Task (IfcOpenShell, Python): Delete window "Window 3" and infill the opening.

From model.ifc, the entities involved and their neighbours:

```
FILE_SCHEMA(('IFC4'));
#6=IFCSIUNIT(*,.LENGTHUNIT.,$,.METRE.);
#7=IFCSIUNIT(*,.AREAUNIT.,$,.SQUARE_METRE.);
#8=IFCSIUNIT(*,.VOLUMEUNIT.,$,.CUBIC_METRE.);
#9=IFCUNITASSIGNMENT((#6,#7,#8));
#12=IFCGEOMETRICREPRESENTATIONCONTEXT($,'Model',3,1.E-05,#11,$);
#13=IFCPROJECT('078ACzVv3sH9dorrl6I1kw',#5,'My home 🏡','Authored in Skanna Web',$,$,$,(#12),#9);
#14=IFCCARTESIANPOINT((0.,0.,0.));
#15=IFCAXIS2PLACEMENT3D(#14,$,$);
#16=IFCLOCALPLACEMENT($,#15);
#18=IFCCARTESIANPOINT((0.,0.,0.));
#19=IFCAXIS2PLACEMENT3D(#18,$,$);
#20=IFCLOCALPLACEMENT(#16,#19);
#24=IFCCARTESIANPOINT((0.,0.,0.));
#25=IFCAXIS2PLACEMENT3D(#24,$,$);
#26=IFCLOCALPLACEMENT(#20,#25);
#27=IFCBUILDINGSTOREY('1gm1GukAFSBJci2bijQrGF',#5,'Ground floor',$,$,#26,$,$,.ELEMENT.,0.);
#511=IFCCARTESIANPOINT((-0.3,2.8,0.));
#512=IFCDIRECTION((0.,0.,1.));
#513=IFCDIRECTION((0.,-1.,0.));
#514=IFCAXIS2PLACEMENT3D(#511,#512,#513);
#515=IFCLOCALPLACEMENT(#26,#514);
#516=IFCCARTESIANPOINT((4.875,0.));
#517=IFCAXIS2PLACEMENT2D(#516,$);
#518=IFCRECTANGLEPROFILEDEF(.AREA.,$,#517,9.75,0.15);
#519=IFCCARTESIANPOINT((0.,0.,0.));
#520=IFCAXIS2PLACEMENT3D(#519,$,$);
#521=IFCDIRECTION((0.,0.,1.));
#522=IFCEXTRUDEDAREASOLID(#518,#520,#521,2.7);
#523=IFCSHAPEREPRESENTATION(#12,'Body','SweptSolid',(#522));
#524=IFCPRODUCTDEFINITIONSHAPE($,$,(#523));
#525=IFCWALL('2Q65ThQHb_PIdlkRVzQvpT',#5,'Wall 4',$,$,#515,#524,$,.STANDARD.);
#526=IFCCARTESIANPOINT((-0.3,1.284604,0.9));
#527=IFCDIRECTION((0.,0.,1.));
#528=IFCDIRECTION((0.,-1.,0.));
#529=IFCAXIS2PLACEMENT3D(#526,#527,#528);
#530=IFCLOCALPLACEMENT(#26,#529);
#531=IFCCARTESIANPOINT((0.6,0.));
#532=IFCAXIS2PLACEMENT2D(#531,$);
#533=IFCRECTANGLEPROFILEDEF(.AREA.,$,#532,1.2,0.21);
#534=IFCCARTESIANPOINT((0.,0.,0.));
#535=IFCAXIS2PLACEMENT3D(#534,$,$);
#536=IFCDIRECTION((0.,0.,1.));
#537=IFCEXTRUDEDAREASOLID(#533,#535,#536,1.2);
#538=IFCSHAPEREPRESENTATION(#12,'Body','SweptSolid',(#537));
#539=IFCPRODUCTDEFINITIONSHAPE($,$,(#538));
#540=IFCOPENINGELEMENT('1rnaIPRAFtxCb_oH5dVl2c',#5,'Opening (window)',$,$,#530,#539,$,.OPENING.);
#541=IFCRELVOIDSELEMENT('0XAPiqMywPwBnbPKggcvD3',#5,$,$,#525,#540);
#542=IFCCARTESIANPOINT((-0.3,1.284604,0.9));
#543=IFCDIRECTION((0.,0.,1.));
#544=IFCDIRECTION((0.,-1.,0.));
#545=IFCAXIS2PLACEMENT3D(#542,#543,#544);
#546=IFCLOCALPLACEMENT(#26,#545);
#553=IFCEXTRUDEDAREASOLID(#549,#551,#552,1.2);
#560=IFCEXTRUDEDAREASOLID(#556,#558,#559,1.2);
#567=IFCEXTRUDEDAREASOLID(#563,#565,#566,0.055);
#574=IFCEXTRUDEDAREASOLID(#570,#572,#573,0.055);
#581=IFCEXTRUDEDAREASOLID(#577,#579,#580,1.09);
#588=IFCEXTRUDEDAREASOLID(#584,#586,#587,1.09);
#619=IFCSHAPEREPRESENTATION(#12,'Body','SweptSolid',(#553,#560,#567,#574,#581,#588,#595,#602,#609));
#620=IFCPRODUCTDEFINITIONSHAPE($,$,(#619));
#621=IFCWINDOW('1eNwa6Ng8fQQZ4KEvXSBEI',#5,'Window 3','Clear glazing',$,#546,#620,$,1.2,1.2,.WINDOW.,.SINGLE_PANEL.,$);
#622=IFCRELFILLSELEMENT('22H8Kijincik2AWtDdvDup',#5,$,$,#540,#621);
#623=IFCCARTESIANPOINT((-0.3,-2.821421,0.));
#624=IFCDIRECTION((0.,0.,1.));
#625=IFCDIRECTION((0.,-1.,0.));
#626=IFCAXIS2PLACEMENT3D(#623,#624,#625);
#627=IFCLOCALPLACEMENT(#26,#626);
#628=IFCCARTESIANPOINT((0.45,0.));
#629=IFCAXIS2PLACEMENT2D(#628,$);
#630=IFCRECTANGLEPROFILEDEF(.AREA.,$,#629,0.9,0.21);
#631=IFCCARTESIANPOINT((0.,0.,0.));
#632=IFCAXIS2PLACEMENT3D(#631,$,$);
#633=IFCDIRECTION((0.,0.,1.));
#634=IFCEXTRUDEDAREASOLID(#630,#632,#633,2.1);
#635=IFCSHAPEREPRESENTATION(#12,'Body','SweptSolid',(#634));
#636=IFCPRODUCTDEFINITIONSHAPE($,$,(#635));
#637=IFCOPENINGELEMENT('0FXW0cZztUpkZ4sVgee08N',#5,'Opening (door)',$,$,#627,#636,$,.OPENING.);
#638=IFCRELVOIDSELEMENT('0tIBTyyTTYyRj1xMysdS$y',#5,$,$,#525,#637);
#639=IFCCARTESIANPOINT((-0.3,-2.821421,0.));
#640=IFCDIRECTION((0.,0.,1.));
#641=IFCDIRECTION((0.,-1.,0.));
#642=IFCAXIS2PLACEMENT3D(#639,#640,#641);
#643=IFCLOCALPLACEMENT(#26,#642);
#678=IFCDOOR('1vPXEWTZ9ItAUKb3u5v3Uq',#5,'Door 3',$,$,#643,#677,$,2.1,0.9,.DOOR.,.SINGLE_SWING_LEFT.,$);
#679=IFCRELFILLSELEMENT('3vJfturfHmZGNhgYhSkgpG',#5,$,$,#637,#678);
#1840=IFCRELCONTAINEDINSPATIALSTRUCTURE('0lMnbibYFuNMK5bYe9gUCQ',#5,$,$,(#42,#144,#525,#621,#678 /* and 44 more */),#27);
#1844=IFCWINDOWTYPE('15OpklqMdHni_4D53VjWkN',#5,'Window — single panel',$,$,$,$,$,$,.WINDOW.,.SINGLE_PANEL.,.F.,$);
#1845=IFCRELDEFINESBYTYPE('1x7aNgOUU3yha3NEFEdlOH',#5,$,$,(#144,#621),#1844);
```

```python
import ifcopenshell
import ifcopenshell.api.feature
import ifcopenshell.api.root
import ifcopenshell.geom
import ifcopenshell.util.shape

model = ifcopenshell.open("model.ifc")
settings = ifcopenshell.geom.settings()


def volume(element):
    """Net volume in cubic metres, openings subtracted."""
    shape = ifcopenshell.geom.create_shape(settings, element)
    return ifcopenshell.util.shape.get_volume(shape.geometry)


window = model.by_id(621)
opening = window.FillsVoids[0].RelatingOpeningElement
wall = opening.VoidsElements[0].RelatingBuildingElement
before = volume(wall)

ifcopenshell.api.root.remove_product(model, product=window)
ifcopenshell.api.feature.remove_feature(model, feature=opening)

after = volume(wall)

print(f"wall volume {before:.3f} -> {after:.3f} m3")

model.write("model-out.ifc")
```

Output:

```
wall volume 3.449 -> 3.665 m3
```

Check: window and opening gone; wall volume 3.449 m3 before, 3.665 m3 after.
